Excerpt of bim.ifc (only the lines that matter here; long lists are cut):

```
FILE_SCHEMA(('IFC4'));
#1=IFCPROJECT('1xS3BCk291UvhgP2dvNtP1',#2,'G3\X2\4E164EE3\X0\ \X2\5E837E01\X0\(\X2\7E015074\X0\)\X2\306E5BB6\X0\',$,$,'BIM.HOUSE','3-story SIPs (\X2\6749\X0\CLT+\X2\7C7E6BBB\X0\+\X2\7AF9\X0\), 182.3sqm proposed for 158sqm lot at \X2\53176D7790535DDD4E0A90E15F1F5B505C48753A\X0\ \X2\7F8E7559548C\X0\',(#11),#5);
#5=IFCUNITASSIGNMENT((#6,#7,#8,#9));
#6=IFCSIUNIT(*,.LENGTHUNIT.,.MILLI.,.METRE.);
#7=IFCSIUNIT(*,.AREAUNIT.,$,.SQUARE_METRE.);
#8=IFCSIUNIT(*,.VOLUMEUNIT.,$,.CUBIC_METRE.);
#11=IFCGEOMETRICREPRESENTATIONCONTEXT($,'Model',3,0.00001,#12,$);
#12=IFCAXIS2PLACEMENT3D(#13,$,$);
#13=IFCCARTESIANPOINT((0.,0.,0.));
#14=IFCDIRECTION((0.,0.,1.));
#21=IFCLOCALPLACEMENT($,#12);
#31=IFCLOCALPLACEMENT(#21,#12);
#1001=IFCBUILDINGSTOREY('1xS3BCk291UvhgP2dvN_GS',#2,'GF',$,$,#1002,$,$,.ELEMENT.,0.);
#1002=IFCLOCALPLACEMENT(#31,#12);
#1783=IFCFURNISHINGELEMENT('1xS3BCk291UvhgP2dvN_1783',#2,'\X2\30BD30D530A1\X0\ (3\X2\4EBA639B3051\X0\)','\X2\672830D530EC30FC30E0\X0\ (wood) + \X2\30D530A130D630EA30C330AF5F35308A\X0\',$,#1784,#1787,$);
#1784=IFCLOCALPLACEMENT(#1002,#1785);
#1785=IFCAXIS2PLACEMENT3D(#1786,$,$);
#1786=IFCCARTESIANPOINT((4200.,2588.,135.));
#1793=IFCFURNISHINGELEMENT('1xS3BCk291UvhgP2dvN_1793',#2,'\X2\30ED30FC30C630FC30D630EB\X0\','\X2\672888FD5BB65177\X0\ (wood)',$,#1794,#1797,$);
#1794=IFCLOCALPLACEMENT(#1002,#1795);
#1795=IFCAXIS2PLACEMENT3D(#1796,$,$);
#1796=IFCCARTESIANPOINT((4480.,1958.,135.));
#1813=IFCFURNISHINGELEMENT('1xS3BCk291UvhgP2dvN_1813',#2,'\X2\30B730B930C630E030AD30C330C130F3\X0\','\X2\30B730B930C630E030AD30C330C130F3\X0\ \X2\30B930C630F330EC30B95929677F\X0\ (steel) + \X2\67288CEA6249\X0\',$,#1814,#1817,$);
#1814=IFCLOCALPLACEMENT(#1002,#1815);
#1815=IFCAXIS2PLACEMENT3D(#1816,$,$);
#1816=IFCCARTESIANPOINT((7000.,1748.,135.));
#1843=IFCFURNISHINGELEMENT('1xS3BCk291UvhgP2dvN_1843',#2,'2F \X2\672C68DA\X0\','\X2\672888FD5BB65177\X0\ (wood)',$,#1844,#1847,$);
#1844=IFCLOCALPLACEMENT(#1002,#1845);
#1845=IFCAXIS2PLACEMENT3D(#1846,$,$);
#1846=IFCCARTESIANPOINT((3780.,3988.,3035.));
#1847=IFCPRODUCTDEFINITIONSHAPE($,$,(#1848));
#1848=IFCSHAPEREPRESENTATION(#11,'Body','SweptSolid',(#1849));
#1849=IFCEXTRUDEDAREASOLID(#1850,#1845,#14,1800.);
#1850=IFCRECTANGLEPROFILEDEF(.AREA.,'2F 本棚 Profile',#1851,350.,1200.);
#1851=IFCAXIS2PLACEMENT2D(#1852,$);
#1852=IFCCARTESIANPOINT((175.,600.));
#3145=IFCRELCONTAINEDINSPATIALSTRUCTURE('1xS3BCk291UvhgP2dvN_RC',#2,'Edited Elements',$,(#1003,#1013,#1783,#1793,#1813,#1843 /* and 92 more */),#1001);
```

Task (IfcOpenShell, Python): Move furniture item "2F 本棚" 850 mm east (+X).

```python
import ifcopenshell
import ifcopenshell.api.geometry
import ifcopenshell.util.placement
import ifcopenshell.util.unit

model = ifcopenshell.open("bim.ifc")
unit_scale = ifcopenshell.util.unit.calculate_unit_scale(model)

item = model.by_id(1843)
matrix = ifcopenshell.util.placement.get_local_placement(item.ObjectPlacement)
matrix[0, 3] += 0.85 / unit_scale
ifcopenshell.api.geometry.edit_object_placement(model, product=item, matrix=matrix, is_si=False)

print(ifcopenshell.util.placement.get_local_placement(item.ObjectPlacement).round(3) + 0.0)

model.write("bim_v2.ifc")
```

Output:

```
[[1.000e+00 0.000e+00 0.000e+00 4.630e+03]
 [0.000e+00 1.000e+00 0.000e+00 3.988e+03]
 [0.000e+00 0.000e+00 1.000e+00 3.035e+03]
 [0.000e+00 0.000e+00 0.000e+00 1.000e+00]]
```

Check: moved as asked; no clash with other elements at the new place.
